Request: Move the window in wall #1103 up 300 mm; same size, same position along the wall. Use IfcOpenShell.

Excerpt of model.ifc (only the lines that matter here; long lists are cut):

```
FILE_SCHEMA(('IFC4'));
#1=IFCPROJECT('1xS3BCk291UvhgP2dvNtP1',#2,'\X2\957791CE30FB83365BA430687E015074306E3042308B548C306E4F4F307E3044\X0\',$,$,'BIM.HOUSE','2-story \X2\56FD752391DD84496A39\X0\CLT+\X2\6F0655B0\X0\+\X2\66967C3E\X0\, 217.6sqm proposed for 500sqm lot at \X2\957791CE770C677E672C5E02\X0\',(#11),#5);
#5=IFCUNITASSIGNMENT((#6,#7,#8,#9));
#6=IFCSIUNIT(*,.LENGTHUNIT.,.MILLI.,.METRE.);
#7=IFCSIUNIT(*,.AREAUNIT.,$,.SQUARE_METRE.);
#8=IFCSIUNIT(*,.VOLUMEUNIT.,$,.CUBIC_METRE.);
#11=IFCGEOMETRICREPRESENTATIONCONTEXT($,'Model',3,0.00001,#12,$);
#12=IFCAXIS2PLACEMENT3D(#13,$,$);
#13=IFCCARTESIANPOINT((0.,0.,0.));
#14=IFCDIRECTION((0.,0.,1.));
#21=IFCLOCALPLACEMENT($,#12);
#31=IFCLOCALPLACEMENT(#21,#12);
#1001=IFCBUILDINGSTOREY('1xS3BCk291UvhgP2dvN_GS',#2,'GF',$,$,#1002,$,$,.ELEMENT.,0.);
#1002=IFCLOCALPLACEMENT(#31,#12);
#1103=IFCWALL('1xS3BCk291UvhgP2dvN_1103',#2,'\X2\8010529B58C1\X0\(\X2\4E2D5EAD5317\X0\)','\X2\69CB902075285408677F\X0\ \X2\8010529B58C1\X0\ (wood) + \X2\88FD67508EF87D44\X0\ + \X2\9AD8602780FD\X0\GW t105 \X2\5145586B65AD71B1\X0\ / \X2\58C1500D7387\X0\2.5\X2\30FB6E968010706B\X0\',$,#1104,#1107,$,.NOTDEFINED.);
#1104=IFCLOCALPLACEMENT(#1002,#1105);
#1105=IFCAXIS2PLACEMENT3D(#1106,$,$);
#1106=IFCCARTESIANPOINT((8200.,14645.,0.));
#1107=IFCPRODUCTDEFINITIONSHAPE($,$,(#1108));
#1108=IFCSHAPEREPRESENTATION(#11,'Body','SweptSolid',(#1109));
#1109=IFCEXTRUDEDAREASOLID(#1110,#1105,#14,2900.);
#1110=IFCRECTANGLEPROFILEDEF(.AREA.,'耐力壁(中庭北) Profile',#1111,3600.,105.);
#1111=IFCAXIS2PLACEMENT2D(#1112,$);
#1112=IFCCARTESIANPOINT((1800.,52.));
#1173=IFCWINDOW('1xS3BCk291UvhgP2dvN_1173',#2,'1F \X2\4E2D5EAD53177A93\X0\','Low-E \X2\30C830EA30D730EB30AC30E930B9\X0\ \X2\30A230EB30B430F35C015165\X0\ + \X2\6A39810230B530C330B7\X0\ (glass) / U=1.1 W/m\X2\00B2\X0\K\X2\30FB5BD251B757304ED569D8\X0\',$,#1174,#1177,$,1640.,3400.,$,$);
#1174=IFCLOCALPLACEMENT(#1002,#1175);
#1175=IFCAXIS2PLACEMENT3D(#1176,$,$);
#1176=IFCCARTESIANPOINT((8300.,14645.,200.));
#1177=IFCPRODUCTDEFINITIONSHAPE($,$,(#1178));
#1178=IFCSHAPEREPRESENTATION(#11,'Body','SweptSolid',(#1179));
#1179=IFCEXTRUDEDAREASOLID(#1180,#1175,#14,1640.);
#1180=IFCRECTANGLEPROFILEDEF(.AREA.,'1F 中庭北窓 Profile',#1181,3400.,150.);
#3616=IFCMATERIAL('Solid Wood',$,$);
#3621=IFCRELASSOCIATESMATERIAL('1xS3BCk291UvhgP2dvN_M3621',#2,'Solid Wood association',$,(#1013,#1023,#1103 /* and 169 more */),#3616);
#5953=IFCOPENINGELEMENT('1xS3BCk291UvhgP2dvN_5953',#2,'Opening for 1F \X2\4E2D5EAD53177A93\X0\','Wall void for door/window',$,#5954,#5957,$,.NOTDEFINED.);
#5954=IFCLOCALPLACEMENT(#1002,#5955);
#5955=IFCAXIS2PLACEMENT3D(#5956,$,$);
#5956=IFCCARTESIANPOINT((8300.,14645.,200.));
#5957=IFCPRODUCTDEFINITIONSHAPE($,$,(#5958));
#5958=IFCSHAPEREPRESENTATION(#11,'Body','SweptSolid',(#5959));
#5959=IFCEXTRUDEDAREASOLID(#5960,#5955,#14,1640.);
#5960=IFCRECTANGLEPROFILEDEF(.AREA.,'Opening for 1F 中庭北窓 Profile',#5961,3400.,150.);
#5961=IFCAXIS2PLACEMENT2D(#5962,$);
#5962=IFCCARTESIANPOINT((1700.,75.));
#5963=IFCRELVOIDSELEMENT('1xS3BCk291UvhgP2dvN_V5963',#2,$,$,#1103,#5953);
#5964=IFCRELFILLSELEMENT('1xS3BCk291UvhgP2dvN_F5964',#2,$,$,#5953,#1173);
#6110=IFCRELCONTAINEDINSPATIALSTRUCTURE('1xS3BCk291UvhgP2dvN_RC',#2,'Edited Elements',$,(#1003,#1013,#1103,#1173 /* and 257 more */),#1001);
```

```python
import numpy as np
import ifcopenshell
import ifcopenshell.api.geometry
import ifcopenshell.util.placement
import ifcopenshell.util.unit

model = ifcopenshell.open("model.ifc")
unit_scale = ifcopenshell.util.unit.calculate_unit_scale(model)

window = model.by_id(1173)
opening = window.FillsVoids[0].RelatingOpeningElement
dz = 0.3 / unit_scale

shift = np.array([0.0, 0.0, dz])
# The window is not placed relative to its opening, so move both.
for product in (opening, window):
    matrix = ifcopenshell.util.placement.get_local_placement(product.ObjectPlacement)
    matrix[:3, 3] += shift
    ifcopenshell.api.geometry.edit_object_placement(model, product=product, matrix=matrix, is_si=False)

print(f"moved by {dz * unit_scale:+.3f} m")

model.write("model_v2.ifc")
```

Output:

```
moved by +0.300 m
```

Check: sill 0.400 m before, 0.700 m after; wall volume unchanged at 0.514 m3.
